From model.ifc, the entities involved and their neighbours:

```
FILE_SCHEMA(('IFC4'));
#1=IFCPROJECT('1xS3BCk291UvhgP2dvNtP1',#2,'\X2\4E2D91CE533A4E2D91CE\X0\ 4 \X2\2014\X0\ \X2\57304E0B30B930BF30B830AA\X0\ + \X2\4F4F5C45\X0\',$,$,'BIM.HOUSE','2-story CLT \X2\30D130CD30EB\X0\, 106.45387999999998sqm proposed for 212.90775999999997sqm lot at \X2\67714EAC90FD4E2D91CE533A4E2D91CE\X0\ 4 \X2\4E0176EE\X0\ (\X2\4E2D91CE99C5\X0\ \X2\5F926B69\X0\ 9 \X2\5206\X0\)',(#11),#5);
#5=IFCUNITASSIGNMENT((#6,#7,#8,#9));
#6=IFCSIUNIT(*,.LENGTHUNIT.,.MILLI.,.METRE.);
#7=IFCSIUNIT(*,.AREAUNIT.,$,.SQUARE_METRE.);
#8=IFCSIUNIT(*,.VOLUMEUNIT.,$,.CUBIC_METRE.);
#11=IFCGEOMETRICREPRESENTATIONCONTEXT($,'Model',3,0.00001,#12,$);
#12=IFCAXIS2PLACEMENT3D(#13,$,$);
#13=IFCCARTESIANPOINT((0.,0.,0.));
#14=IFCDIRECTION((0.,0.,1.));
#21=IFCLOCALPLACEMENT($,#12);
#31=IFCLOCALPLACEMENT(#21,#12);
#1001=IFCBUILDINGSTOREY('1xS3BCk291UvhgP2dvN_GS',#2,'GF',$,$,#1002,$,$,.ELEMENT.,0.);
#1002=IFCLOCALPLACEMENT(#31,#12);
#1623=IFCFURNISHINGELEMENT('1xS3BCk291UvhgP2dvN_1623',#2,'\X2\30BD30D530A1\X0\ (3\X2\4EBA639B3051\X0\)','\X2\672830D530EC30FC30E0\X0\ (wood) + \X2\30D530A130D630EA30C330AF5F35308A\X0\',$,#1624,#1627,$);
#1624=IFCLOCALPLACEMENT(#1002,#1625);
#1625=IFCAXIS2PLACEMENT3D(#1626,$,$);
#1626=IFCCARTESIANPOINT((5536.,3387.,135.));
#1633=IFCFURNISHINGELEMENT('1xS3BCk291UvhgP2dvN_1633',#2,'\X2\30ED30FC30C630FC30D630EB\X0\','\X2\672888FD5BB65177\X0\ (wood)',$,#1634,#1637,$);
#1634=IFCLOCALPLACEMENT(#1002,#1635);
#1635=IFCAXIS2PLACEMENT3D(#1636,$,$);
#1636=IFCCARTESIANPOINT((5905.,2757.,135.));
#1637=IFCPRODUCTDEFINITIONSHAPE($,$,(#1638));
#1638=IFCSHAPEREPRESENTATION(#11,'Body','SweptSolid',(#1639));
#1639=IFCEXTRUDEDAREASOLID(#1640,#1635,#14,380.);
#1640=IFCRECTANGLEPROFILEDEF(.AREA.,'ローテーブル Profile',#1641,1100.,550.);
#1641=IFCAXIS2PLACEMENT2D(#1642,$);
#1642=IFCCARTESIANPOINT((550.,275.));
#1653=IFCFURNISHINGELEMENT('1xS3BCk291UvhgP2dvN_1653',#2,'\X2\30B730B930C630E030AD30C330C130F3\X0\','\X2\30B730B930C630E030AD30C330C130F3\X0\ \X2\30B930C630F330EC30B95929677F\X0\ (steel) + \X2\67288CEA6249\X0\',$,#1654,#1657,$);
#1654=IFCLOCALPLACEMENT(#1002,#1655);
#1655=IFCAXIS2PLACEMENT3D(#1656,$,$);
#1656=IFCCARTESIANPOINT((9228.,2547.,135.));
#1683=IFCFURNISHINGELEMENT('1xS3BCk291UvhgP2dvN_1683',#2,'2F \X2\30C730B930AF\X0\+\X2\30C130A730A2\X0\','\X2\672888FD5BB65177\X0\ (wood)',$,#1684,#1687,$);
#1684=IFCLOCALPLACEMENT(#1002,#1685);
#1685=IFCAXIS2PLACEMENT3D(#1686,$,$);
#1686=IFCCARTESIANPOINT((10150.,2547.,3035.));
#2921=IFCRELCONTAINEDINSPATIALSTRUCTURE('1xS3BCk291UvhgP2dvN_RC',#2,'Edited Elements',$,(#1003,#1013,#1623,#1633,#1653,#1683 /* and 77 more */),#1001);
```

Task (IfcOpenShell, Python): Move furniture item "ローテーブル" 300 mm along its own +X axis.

```python
import ifcopenshell
import ifcopenshell.api.geometry
import ifcopenshell.util.placement
import ifcopenshell.util.unit

model = ifcopenshell.open("model.ifc")
unit_scale = ifcopenshell.util.unit.calculate_unit_scale(model)

item = model.by_guid("1xS3BCk291UvhgP2dvN_1633")
matrix = ifcopenshell.util.placement.get_local_placement(item.ObjectPlacement)
matrix[:3, 3] += matrix[:3, 0] * 0.3 / unit_scale
ifcopenshell.api.geometry.edit_object_placement(model, product=item, matrix=matrix, is_si=False)

print(ifcopenshell.util.placement.get_local_placement(item.ObjectPlacement).round(3) + 0.0)

model.write("model_v2.ifc")
```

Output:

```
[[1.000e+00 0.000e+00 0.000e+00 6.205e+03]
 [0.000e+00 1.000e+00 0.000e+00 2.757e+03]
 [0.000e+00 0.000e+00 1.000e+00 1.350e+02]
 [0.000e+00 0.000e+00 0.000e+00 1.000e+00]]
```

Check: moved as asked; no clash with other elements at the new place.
